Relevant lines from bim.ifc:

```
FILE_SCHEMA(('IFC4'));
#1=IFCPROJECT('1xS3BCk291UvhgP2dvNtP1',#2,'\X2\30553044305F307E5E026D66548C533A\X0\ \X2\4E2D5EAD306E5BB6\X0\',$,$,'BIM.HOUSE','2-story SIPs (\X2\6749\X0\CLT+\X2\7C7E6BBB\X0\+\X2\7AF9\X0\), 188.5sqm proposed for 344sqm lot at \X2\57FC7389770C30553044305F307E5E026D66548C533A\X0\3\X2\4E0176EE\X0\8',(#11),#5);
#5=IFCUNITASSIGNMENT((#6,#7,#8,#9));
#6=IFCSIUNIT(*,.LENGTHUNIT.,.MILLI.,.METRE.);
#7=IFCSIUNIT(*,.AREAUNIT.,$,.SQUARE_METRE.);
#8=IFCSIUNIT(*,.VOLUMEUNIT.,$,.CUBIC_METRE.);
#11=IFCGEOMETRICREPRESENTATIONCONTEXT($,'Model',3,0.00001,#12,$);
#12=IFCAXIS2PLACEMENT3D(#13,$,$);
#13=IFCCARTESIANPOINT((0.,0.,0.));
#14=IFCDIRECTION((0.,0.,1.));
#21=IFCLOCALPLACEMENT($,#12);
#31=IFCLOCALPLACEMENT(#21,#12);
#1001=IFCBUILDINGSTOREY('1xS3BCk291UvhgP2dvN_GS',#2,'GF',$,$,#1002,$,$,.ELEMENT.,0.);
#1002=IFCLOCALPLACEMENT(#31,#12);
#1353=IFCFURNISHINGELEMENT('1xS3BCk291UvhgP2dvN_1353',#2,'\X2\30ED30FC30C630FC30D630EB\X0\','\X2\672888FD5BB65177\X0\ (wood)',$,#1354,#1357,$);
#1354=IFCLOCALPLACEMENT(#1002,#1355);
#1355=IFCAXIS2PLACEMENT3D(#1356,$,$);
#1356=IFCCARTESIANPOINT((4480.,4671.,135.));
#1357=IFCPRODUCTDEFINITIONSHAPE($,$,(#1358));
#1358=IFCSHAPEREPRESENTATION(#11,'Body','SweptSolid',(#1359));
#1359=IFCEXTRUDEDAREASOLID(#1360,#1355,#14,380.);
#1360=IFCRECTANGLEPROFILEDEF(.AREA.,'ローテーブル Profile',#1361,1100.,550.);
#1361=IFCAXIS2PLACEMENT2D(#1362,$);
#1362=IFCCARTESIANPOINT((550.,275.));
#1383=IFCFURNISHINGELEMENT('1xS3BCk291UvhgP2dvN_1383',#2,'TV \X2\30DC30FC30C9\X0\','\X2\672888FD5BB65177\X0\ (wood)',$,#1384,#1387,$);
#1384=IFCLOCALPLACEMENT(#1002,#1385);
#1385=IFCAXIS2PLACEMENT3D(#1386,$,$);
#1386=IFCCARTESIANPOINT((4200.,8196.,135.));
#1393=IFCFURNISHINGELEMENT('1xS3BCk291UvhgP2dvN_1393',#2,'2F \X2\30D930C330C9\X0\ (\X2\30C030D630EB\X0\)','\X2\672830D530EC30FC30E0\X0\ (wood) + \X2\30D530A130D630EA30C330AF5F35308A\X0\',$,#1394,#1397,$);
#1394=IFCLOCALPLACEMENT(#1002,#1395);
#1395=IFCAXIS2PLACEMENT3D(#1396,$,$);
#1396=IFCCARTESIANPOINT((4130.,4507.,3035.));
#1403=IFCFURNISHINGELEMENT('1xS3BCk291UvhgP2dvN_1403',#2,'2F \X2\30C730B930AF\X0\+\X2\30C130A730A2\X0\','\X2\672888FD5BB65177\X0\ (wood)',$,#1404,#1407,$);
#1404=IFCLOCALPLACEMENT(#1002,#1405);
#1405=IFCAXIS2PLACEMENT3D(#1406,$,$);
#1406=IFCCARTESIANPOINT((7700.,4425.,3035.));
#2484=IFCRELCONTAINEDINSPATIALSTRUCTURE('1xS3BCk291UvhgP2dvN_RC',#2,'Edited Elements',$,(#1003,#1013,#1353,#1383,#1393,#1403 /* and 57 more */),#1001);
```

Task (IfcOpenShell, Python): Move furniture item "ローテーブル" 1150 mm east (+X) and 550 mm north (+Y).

```python
import ifcopenshell
import ifcopenshell.api.geometry
import ifcopenshell.util.placement
import ifcopenshell.util.unit

model = ifcopenshell.open("bim.ifc")
unit_scale = ifcopenshell.util.unit.calculate_unit_scale(model)

item = model.by_guid("1xS3BCk291UvhgP2dvN_1353")
matrix = ifcopenshell.util.placement.get_local_placement(item.ObjectPlacement)
matrix[0, 3] += 1.15 / unit_scale
matrix[1, 3] += 0.55 / unit_scale
ifcopenshell.api.geometry.edit_object_placement(model, product=item, matrix=matrix, is_si=False)

print(ifcopenshell.util.placement.get_local_placement(item.ObjectPlacement).round(3) + 0.0)

model.write("bim_updated.ifc")
```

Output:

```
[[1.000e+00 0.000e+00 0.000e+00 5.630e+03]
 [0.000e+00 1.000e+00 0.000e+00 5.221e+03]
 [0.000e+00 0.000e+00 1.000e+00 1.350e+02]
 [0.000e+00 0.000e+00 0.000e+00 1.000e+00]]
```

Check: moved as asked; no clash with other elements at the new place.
